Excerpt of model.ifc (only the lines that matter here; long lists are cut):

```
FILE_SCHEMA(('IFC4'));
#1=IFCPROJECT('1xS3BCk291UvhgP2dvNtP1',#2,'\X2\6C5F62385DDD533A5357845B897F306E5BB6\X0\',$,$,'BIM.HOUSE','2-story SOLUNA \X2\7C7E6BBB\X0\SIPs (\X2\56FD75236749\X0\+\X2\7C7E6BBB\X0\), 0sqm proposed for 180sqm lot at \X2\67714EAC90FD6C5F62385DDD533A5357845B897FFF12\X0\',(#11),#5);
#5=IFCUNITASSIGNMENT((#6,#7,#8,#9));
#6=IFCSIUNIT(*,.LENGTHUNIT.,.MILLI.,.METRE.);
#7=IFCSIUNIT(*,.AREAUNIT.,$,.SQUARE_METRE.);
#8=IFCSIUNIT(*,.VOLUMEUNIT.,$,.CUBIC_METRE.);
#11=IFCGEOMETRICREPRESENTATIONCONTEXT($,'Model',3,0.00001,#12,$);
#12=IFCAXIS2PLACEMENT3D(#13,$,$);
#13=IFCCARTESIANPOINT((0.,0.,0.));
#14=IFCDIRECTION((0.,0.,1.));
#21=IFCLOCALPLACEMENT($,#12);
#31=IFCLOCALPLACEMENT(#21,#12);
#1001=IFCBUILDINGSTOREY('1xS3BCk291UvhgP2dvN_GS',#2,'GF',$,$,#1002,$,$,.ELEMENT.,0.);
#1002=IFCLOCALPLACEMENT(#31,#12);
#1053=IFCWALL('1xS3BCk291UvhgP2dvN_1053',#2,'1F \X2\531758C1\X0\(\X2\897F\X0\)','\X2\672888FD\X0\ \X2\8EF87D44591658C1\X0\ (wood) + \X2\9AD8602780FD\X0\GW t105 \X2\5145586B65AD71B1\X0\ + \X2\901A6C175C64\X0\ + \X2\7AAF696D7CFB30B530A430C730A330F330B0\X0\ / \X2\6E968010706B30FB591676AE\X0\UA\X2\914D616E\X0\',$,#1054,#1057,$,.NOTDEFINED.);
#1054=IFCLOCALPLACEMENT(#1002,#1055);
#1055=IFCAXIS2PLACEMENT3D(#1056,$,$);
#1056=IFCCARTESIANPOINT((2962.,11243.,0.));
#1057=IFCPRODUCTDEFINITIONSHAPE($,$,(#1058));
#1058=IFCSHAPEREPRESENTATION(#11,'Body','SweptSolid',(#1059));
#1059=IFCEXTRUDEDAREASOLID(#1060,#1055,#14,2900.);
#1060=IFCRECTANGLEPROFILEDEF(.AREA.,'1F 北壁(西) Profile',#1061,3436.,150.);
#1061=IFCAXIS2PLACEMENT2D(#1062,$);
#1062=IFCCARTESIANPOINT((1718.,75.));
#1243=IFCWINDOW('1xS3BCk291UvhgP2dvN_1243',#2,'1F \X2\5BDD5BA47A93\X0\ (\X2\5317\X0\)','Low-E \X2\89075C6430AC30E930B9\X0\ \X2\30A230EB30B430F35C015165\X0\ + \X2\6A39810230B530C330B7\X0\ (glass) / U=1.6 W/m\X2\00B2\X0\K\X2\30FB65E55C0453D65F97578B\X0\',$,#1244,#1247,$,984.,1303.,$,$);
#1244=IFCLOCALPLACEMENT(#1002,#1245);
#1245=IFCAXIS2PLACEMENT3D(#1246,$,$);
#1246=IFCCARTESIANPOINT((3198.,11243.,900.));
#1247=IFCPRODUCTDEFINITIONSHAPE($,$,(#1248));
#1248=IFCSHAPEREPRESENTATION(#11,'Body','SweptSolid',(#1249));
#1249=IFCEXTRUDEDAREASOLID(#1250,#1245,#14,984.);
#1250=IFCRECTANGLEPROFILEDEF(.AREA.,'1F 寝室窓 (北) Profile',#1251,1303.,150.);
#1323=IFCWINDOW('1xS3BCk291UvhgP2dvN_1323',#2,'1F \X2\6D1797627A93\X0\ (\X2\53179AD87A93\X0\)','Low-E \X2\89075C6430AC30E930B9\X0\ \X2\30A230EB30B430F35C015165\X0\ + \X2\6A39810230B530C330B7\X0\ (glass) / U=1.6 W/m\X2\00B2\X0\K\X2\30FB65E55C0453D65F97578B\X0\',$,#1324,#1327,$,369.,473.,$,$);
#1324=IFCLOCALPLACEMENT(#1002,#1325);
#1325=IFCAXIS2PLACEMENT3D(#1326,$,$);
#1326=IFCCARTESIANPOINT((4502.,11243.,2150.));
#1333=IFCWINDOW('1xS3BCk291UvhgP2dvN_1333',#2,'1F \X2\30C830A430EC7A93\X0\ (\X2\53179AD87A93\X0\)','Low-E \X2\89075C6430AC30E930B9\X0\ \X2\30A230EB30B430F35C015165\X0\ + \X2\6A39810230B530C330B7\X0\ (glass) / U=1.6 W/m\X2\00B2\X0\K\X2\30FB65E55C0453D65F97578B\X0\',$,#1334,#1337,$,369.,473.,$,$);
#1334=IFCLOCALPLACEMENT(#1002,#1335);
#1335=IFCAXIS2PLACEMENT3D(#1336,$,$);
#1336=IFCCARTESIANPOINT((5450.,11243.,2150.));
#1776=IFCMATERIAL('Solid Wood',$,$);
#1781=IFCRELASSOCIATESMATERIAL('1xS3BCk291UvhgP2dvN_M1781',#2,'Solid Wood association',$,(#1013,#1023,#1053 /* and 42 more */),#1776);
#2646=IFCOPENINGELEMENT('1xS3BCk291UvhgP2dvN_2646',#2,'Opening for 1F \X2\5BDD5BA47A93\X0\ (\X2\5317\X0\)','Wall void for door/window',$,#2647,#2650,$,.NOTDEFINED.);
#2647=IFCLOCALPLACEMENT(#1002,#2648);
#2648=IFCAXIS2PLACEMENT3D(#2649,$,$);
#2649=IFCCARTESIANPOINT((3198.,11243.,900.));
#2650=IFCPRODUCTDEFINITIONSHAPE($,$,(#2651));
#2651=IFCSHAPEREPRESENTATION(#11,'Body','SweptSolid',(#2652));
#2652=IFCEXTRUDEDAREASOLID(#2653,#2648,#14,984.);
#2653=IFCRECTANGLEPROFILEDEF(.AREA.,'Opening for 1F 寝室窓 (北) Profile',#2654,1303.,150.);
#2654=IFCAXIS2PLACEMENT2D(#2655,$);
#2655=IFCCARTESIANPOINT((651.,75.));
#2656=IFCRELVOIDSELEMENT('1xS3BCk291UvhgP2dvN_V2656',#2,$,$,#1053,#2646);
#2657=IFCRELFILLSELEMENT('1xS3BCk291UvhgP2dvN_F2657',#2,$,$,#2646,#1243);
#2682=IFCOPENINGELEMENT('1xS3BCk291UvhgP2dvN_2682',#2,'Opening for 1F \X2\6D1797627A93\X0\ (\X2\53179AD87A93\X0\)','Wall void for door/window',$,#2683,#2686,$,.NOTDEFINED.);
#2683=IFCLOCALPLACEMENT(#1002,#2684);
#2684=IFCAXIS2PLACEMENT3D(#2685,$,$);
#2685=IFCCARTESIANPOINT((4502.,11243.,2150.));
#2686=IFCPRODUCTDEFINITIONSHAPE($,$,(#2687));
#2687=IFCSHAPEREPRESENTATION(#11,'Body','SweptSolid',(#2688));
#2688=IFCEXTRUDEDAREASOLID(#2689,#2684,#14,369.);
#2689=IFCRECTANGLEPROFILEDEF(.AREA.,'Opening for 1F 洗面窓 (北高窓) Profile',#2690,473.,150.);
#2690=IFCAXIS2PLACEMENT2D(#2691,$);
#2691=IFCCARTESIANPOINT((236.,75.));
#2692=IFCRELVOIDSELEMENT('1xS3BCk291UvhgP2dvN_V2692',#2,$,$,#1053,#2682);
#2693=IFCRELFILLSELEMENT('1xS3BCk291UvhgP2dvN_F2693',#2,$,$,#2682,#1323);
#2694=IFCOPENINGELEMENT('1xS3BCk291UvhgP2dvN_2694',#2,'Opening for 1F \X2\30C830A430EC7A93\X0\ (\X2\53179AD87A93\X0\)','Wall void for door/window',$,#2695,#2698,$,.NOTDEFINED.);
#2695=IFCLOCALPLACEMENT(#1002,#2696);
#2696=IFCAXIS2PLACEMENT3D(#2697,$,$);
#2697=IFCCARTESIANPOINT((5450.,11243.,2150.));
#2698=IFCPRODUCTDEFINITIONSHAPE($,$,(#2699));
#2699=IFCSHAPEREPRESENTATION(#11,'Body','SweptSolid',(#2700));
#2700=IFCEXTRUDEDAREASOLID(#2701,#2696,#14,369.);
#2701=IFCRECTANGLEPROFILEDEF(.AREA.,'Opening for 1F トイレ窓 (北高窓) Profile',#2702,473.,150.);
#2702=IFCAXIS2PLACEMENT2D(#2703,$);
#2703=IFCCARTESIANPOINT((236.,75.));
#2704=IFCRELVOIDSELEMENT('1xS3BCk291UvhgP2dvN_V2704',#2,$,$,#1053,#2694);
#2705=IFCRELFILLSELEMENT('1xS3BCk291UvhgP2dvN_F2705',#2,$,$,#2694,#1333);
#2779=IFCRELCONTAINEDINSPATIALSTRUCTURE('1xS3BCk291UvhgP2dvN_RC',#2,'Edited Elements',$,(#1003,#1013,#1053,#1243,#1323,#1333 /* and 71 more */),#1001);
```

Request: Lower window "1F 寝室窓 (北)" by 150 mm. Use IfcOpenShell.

```python
import numpy as np
import ifcopenshell
import ifcopenshell.api.geometry
import ifcopenshell.util.placement
import ifcopenshell.util.unit

model = ifcopenshell.open("model.ifc")
unit_scale = ifcopenshell.util.unit.calculate_unit_scale(model)

window = model.by_guid("1xS3BCk291UvhgP2dvN_1243")
opening = window.FillsVoids[0].RelatingOpeningElement
dz = -0.15 / unit_scale

shift = np.array([0.0, 0.0, dz])
# The window is not placed relative to its opening, so move both.
for product in (opening, window):
    matrix = ifcopenshell.util.placement.get_local_placement(product.ObjectPlacement)
    matrix[:3, 3] += shift
    ifcopenshell.api.geometry.edit_object_placement(model, product=product, matrix=matrix, is_si=False)

print(f"moved by {dz * unit_scale:+.3f} m")

model.write("model_edited.ifc")
```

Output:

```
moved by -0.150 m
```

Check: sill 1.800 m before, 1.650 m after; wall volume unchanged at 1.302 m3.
